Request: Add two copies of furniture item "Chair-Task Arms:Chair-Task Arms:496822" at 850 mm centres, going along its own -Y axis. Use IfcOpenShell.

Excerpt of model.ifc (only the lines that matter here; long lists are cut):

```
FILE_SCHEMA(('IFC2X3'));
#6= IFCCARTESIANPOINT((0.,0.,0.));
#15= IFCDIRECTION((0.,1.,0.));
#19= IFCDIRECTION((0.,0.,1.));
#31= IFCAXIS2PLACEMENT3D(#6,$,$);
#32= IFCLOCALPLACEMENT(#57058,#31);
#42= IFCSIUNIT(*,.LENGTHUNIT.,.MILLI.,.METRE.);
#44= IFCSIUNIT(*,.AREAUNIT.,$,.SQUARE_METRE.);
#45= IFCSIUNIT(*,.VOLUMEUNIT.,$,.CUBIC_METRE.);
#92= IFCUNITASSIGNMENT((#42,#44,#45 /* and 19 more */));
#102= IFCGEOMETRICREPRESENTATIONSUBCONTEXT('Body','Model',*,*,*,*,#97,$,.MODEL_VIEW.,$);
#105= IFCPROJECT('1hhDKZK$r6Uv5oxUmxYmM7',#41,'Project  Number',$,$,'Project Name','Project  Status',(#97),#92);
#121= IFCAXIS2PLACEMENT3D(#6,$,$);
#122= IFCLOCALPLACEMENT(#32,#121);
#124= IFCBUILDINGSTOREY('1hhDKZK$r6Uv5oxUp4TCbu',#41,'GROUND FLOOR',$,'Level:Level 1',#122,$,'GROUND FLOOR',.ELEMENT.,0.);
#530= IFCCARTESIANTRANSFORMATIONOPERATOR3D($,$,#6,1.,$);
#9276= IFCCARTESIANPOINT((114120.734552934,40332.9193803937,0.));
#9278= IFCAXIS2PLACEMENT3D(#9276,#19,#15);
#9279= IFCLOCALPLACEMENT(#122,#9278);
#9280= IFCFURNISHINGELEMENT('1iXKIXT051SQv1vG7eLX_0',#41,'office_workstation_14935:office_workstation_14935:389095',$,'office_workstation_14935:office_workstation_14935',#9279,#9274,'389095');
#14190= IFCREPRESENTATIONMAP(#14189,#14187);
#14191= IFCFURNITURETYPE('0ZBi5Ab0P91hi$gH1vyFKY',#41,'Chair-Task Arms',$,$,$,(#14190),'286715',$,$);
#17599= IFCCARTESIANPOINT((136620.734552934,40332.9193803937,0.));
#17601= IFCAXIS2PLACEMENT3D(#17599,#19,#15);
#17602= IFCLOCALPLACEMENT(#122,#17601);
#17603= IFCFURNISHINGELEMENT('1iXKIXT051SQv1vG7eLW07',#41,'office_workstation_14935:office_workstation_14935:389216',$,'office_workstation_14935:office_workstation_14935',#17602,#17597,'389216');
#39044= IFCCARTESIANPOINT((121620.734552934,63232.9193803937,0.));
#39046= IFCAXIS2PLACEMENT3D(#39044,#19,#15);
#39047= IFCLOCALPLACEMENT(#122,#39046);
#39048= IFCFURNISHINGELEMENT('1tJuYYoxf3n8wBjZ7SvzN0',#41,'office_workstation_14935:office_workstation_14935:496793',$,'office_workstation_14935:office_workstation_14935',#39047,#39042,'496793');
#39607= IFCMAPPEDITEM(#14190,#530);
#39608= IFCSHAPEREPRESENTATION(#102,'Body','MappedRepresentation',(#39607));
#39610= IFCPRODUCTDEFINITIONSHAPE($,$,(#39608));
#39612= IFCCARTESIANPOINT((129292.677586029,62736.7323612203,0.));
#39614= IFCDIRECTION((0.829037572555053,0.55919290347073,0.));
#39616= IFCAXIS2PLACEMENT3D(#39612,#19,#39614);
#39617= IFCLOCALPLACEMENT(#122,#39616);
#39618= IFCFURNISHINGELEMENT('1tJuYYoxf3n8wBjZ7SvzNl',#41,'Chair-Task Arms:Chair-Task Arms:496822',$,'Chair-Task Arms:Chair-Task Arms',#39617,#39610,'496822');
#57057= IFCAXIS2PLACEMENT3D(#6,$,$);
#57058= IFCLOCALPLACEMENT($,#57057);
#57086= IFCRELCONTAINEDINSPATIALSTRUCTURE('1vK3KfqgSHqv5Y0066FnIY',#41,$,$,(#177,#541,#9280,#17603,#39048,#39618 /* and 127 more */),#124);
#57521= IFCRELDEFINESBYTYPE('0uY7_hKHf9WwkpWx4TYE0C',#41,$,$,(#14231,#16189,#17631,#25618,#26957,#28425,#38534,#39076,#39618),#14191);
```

```python
import ifcopenshell
import ifcopenshell.api.geometry
import ifcopenshell.api.root
import ifcopenshell.util.element
import ifcopenshell.util.placement
import ifcopenshell.util.unit

model = ifcopenshell.open("model.ifc")
unit_scale = ifcopenshell.util.unit.calculate_unit_scale(model)


def reuse_history(source, copy):
    """copy_class also copies each property set's owner history, people and application; keep the originals."""
    for rel in copy.IsDefinedBy:
        if rel.is_a("IfcRelDefinesByProperties") and (history := rel.RelatingPropertyDefinition.OwnerHistory):
            rel.RelatingPropertyDefinition.OwnerHistory = source.OwnerHistory
            ifcopenshell.util.element.remove_deep2(model, history)


source = model.by_guid("1tJuYYoxf3n8wBjZ7SvzNl")
base = ifcopenshell.util.placement.get_local_placement(source.ObjectPlacement)
step = -base[:3, 1] * 0.85 / unit_scale

for i in range(1, 3):
    copy = ifcopenshell.api.root.copy_class(model, product=source)
    copy.Representation = ifcopenshell.util.element.copy_deep(
        model, source.Representation, exclude=["IfcGeometricRepresentationContext", "IfcRepresentationMap"]
    )
    copy.Name = "Chair-Task Arms:Chair-Task Arms"
    copy.Tag = None
    reuse_history(source, copy)
    matrix = base.copy()
    matrix[:3, 3] += i * step
    print("added at", matrix[:3, 3].round(3) + 0.0)
    ifcopenshell.api.geometry.edit_object_placement(model, product=copy, matrix=matrix, is_si=False)

model.write("model-out.ifc")
```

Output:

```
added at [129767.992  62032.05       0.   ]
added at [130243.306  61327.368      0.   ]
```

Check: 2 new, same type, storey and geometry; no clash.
